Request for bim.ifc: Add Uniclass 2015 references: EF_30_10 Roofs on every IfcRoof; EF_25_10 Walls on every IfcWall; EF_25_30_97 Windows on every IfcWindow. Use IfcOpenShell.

First a look at what the model holds.

```python
import ifcopenshell

model = ifcopenshell.open("bim.ifc")
print(model.schema)
print("classifications:", [c.Name for c in model.by_type("IfcClassification")])
for ifc_class in ("IfcDoor", "IfcRoof", "IfcStair", "IfcWall", "IfcWindow"):
    print(ifc_class, len(model.by_type(ifc_class)))
```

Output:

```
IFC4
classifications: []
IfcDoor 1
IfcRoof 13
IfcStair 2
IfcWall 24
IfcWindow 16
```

```python
import ifcopenshell
import ifcopenshell.api.classification

model = ifcopenshell.open("bim.ifc")

system = ifcopenshell.api.classification.add_classification(model, classification="Uniclass 2015")

codes = {
    "IfcRoof": ("EF_30_10", "Roofs"),
    "IfcWall": ("EF_25_10", "Walls"),
    "IfcWindow": ("EF_25_30_97", "Windows"),
}
for ifc_class, (code, name) in codes.items():
    products = model.by_type(ifc_class)
    ifcopenshell.api.classification.add_reference(
        model, products=products, classification=system, identification=code, name=name
    )
    print(code, len(products))

model.write("bim-out.ifc")
```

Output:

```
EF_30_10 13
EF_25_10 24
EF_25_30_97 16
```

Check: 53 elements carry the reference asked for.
